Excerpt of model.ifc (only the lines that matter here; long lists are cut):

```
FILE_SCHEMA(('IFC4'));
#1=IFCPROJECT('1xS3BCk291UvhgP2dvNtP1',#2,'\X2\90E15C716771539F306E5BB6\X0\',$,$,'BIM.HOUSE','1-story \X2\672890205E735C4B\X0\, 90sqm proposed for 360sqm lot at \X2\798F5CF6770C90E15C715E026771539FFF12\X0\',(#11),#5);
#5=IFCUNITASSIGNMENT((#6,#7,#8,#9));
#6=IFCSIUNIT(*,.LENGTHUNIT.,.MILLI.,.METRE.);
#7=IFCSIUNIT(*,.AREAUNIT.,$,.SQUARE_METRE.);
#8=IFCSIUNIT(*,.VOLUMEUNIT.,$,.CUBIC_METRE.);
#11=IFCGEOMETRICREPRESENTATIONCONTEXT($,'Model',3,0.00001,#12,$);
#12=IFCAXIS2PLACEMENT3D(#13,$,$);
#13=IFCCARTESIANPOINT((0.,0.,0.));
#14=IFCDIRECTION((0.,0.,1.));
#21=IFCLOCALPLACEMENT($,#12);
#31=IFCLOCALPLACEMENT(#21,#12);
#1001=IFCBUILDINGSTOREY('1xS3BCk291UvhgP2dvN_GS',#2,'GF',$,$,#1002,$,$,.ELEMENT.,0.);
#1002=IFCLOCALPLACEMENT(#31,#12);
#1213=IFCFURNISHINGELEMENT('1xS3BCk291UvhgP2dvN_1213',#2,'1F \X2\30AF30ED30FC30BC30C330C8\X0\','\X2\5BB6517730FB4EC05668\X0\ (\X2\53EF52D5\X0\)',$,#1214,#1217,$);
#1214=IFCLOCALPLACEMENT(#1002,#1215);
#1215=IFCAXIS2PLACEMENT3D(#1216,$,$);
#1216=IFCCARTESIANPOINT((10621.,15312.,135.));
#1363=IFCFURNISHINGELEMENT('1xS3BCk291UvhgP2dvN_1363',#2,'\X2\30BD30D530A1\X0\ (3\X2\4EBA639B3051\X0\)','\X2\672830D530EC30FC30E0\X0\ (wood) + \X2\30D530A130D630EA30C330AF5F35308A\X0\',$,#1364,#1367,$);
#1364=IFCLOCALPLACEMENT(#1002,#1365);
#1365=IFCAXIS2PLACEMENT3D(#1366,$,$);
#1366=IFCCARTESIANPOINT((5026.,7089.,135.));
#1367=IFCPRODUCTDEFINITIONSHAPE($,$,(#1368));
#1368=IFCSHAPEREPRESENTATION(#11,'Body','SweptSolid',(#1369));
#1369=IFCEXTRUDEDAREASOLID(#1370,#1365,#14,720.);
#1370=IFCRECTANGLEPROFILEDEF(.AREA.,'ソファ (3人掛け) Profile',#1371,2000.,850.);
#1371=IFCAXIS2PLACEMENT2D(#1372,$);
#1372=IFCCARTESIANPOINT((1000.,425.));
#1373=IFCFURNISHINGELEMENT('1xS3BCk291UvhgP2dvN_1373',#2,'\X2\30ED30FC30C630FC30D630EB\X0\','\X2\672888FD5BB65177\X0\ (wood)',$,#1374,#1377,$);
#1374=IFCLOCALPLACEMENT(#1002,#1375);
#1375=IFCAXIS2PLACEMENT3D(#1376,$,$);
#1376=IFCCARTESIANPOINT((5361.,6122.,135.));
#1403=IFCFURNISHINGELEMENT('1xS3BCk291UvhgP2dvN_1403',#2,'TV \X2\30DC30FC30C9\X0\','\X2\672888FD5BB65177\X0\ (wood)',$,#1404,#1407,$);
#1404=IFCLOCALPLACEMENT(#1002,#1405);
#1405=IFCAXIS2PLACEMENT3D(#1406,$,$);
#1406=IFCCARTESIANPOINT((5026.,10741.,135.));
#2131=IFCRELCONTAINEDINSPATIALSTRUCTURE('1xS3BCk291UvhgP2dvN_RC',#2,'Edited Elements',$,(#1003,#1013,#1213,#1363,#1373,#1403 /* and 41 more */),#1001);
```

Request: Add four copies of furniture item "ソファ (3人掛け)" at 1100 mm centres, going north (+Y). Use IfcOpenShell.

```python
import numpy as np
import ifcopenshell
import ifcopenshell.api.geometry
import ifcopenshell.api.root
import ifcopenshell.util.element
import ifcopenshell.util.placement
import ifcopenshell.util.unit

model = ifcopenshell.open("model.ifc")
unit_scale = ifcopenshell.util.unit.calculate_unit_scale(model)


def reuse_history(source, copy):
    """copy_class also copies each property set's owner history, people and application; keep the originals."""
    for rel in copy.IsDefinedBy:
        if rel.is_a("IfcRelDefinesByProperties") and (history := rel.RelatingPropertyDefinition.OwnerHistory):
            rel.RelatingPropertyDefinition.OwnerHistory = source.OwnerHistory
            ifcopenshell.util.element.remove_deep2(model, history)


source = model.by_guid("1xS3BCk291UvhgP2dvN_1363")
base = ifcopenshell.util.placement.get_local_placement(source.ObjectPlacement)
step = np.array([0.0, 1.0, 0.0]) * 1.1 / unit_scale

for i in range(1, 5):
    copy = ifcopenshell.api.root.copy_class(model, product=source)
    copy.Representation = ifcopenshell.util.element.copy_deep(
        model, source.Representation, exclude=["IfcGeometricRepresentationContext", "IfcRepresentationMap"]
    )
    reuse_history(source, copy)
    matrix = base.copy()
    matrix[:3, 3] += i * step
    print("added at", matrix[:3, 3].round(3) + 0.0)
    ifcopenshell.api.geometry.edit_object_placement(model, product=copy, matrix=matrix, is_si=False)

model.write("model_rev.ifc")
```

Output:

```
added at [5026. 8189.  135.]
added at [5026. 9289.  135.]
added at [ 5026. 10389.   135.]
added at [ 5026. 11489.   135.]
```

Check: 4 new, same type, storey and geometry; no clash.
